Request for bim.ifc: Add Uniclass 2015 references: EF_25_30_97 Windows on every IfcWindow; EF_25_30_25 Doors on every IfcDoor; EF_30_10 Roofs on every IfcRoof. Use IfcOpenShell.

First a look at what the model holds.

```python
import ifcopenshell

model = ifcopenshell.open("bim.ifc")
print(model.schema)
print("classifications:", [c.Name for c in model.by_type("IfcClassification")])
for ifc_class in ("IfcDoor", "IfcRoof", "IfcStair", "IfcWall", "IfcWindow"):
    print(ifc_class, len(model.by_type(ifc_class)))
```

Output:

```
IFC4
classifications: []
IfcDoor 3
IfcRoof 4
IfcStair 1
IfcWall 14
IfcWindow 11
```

```python
import ifcopenshell
import ifcopenshell.api.classification

model = ifcopenshell.open("bim.ifc")

system = ifcopenshell.api.classification.add_classification(model, classification="Uniclass 2015")

codes = {
    "IfcWindow": ("EF_25_30_97", "Windows"),
    "IfcDoor": ("EF_25_30_25", "Doors"),
    "IfcRoof": ("EF_30_10", "Roofs"),
}
for ifc_class, (code, name) in codes.items():
    products = model.by_type(ifc_class)
    ifcopenshell.api.classification.add_reference(
        model, products=products, classification=system, identification=code, name=name
    )
    print(code, len(products))

model.write("bim_updated.ifc")
```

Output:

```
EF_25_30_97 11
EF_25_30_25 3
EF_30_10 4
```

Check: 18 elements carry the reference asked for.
